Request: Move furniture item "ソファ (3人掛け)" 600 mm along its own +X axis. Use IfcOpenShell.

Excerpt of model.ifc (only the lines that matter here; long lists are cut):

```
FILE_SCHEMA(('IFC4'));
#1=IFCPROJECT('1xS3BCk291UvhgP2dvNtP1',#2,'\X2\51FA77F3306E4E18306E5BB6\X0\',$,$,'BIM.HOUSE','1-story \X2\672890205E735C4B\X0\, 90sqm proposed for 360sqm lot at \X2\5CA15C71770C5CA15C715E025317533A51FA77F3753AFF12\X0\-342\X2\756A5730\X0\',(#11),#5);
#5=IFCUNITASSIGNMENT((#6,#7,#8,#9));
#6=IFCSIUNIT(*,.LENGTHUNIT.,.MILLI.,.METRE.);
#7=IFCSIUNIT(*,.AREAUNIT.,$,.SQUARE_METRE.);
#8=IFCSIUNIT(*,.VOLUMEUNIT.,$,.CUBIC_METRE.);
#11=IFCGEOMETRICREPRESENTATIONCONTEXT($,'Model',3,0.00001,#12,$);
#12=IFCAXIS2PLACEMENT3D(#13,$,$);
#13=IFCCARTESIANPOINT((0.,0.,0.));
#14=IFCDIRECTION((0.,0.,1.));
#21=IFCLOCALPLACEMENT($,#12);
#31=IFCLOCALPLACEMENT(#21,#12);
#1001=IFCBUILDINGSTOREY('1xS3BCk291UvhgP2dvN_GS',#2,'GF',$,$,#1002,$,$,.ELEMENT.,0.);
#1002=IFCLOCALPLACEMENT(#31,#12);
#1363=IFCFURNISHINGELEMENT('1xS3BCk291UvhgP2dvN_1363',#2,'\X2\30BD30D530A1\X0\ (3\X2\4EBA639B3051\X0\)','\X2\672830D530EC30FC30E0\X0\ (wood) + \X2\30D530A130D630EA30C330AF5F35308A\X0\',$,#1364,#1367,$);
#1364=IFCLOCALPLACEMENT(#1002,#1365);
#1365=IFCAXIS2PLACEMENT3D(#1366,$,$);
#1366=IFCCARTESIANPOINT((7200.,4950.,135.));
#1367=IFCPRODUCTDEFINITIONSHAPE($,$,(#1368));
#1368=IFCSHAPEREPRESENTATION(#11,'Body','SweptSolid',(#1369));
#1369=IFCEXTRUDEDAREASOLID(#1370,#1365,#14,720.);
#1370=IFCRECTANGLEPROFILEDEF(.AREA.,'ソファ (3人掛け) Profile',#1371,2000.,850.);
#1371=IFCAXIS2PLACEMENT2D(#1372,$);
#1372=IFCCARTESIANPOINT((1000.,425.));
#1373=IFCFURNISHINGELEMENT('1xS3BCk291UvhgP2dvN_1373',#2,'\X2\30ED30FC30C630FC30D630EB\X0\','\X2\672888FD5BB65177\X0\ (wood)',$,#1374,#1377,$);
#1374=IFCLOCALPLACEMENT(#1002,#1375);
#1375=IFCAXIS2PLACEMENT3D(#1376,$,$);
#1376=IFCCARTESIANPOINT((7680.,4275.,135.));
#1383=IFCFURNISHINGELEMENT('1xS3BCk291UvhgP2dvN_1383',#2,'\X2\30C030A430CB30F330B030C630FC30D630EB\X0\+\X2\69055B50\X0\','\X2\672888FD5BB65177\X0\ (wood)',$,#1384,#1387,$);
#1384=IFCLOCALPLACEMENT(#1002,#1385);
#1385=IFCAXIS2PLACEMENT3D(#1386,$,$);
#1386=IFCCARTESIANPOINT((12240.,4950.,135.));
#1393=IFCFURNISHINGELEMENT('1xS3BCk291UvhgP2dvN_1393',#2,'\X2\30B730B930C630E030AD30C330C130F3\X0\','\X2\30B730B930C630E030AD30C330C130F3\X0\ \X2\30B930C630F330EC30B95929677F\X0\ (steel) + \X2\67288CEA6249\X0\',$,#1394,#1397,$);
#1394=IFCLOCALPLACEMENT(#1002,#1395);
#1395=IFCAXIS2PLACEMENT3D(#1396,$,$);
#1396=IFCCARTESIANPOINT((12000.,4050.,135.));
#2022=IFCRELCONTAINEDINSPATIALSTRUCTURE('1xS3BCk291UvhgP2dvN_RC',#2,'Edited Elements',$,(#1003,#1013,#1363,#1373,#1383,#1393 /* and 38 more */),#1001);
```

```python
import ifcopenshell
import ifcopenshell.api.geometry
import ifcopenshell.util.placement
import ifcopenshell.util.unit

model = ifcopenshell.open("model.ifc")
unit_scale = ifcopenshell.util.unit.calculate_unit_scale(model)

item = model.by_guid("1xS3BCk291UvhgP2dvN_1363")
matrix = ifcopenshell.util.placement.get_local_placement(item.ObjectPlacement)
matrix[:3, 3] += matrix[:3, 0] * 0.6 / unit_scale
ifcopenshell.api.geometry.edit_object_placement(model, product=item, matrix=matrix, is_si=False)

print(ifcopenshell.util.placement.get_local_placement(item.ObjectPlacement).round(3) + 0.0)

model.write("model_updated.ifc")
```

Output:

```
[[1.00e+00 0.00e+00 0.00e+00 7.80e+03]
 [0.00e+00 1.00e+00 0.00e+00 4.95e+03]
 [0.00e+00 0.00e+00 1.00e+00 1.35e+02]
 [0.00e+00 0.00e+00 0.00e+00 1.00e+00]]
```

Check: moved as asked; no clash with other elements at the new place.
